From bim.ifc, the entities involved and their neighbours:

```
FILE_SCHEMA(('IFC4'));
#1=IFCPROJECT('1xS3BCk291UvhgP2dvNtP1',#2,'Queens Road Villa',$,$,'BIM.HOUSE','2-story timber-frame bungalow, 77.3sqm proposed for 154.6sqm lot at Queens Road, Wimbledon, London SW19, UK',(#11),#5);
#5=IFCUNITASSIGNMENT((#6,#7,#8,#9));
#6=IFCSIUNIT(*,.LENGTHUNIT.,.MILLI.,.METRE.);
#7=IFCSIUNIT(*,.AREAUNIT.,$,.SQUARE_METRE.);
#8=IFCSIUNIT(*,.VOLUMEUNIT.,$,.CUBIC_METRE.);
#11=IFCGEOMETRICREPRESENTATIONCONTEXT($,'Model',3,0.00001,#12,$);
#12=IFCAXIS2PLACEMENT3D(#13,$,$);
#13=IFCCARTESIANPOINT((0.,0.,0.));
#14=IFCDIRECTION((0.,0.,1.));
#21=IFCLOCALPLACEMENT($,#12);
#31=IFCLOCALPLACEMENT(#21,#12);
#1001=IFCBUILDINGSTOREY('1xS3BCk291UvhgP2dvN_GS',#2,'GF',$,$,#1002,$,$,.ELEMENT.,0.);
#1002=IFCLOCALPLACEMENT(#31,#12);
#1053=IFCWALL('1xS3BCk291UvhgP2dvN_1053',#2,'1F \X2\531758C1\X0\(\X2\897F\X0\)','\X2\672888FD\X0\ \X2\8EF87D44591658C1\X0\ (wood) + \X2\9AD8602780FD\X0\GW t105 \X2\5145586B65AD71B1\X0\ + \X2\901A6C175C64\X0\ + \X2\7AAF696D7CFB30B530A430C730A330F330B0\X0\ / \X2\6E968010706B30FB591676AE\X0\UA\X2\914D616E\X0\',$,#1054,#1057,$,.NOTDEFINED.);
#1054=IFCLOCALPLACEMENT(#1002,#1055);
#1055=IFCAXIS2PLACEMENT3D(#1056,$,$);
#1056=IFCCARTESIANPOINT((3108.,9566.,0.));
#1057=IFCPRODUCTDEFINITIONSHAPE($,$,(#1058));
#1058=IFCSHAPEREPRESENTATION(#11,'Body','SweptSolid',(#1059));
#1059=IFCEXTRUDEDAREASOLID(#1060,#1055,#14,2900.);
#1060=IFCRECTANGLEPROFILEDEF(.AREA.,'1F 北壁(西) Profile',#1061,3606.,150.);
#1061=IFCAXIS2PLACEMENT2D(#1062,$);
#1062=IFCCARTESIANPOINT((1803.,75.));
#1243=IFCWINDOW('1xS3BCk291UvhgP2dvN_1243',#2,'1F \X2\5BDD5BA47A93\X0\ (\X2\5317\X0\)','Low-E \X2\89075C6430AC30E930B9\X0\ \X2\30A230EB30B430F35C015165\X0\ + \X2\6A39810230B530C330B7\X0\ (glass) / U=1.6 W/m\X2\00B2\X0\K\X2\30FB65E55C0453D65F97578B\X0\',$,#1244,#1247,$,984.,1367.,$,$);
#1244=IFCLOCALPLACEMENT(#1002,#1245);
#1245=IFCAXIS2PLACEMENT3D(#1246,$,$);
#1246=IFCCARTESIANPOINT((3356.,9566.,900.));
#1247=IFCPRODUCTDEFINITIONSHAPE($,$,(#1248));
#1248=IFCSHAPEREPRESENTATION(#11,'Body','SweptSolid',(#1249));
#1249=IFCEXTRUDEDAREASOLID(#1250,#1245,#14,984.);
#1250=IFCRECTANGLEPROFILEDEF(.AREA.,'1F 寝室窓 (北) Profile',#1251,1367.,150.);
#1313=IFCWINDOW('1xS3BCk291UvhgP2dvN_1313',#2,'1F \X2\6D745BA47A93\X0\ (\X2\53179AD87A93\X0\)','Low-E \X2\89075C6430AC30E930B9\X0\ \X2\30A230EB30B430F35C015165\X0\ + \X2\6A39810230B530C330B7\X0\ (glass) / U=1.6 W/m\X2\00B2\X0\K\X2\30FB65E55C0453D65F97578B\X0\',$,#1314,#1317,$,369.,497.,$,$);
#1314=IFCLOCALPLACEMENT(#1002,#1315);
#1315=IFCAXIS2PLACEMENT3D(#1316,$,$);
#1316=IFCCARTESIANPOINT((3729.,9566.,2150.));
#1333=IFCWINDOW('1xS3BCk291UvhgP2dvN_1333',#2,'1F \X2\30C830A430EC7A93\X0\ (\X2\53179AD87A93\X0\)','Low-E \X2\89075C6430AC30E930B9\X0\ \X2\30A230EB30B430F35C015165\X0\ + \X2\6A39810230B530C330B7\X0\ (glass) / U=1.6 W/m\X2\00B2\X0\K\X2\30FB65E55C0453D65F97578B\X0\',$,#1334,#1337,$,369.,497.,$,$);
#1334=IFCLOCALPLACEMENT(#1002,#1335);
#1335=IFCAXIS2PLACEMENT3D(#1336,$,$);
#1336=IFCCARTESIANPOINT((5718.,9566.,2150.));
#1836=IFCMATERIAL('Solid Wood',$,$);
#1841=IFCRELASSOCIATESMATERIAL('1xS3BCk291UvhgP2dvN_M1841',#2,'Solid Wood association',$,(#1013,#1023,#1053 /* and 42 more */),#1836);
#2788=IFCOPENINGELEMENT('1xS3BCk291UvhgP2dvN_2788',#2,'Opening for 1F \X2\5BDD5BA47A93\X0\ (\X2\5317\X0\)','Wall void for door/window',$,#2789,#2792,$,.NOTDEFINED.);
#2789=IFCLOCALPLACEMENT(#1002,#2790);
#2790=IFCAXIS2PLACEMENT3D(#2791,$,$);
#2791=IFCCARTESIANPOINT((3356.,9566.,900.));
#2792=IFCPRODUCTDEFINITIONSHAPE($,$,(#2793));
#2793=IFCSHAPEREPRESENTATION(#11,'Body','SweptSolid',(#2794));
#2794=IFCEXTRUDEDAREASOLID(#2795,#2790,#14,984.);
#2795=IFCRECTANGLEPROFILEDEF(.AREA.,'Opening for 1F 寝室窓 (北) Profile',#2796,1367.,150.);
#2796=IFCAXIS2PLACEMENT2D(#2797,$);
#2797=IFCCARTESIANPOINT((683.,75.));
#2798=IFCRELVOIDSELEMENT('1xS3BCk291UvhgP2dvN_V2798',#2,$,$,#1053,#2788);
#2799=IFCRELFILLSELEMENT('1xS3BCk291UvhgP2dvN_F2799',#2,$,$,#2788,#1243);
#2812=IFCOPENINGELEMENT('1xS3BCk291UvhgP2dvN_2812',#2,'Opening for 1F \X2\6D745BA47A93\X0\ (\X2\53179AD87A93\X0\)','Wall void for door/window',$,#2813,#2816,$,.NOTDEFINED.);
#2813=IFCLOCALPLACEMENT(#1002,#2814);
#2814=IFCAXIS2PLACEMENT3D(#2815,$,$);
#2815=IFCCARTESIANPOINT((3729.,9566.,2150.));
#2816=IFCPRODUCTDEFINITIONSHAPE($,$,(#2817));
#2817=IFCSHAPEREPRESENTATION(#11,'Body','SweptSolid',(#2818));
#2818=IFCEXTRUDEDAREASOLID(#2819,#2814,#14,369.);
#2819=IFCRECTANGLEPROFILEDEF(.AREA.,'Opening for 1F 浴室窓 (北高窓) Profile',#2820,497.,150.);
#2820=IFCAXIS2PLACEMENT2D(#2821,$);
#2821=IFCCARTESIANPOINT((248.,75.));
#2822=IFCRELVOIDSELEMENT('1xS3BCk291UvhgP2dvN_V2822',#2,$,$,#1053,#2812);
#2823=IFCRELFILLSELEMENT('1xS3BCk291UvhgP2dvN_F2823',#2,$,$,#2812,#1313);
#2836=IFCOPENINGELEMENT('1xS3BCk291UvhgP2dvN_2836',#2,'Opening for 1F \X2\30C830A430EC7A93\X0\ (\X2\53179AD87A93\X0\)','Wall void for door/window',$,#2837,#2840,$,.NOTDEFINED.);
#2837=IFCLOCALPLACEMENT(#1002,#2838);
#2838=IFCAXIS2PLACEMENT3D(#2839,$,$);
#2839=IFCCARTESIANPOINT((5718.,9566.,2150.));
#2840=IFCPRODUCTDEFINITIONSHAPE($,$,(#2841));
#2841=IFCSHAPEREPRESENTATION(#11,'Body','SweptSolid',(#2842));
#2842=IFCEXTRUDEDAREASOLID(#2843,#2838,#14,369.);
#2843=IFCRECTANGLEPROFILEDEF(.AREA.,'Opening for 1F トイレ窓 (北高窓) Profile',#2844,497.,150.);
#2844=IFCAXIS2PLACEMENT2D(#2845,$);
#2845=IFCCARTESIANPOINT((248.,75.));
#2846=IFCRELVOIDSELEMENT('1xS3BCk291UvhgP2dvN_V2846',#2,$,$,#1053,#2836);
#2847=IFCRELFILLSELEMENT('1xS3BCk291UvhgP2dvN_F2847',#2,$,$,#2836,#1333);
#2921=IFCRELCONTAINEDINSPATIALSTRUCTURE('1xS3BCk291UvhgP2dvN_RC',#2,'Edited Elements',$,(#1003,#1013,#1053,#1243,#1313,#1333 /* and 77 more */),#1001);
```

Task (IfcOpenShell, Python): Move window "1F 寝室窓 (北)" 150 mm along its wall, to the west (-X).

```python
import ifcopenshell
import ifcopenshell.api.geometry
import ifcopenshell.util.placement
import ifcopenshell.util.unit

model = ifcopenshell.open("bim.ifc")
unit_scale = ifcopenshell.util.unit.calculate_unit_scale(model)

window = model.by_guid("1xS3BCk291UvhgP2dvN_1243")
opening = window.FillsVoids[0].RelatingOpeningElement
wall = opening.VoidsElements[0].RelatingBuildingElement

wall_matrix = ifcopenshell.util.placement.get_local_placement(wall.ObjectPlacement)
shift = wall_matrix[:3, 0] * -0.15 / unit_scale
before = ifcopenshell.util.placement.get_local_placement(window.ObjectPlacement)[:3, 3].copy()

# The window is not placed relative to its opening, so move both.
for product in (opening, window):
    matrix = ifcopenshell.util.placement.get_local_placement(product.ObjectPlacement)
    matrix[:3, 3] += shift
    ifcopenshell.api.geometry.edit_object_placement(model, product=product, matrix=matrix, is_si=False)

after = ifcopenshell.util.placement.get_local_placement(window.ObjectPlacement)[:3, 3]
print("window moved by", (after - before).round(3) + 0.0)

model.write("bim_rev.ifc")
```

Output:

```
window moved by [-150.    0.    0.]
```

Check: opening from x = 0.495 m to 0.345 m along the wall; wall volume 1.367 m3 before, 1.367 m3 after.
